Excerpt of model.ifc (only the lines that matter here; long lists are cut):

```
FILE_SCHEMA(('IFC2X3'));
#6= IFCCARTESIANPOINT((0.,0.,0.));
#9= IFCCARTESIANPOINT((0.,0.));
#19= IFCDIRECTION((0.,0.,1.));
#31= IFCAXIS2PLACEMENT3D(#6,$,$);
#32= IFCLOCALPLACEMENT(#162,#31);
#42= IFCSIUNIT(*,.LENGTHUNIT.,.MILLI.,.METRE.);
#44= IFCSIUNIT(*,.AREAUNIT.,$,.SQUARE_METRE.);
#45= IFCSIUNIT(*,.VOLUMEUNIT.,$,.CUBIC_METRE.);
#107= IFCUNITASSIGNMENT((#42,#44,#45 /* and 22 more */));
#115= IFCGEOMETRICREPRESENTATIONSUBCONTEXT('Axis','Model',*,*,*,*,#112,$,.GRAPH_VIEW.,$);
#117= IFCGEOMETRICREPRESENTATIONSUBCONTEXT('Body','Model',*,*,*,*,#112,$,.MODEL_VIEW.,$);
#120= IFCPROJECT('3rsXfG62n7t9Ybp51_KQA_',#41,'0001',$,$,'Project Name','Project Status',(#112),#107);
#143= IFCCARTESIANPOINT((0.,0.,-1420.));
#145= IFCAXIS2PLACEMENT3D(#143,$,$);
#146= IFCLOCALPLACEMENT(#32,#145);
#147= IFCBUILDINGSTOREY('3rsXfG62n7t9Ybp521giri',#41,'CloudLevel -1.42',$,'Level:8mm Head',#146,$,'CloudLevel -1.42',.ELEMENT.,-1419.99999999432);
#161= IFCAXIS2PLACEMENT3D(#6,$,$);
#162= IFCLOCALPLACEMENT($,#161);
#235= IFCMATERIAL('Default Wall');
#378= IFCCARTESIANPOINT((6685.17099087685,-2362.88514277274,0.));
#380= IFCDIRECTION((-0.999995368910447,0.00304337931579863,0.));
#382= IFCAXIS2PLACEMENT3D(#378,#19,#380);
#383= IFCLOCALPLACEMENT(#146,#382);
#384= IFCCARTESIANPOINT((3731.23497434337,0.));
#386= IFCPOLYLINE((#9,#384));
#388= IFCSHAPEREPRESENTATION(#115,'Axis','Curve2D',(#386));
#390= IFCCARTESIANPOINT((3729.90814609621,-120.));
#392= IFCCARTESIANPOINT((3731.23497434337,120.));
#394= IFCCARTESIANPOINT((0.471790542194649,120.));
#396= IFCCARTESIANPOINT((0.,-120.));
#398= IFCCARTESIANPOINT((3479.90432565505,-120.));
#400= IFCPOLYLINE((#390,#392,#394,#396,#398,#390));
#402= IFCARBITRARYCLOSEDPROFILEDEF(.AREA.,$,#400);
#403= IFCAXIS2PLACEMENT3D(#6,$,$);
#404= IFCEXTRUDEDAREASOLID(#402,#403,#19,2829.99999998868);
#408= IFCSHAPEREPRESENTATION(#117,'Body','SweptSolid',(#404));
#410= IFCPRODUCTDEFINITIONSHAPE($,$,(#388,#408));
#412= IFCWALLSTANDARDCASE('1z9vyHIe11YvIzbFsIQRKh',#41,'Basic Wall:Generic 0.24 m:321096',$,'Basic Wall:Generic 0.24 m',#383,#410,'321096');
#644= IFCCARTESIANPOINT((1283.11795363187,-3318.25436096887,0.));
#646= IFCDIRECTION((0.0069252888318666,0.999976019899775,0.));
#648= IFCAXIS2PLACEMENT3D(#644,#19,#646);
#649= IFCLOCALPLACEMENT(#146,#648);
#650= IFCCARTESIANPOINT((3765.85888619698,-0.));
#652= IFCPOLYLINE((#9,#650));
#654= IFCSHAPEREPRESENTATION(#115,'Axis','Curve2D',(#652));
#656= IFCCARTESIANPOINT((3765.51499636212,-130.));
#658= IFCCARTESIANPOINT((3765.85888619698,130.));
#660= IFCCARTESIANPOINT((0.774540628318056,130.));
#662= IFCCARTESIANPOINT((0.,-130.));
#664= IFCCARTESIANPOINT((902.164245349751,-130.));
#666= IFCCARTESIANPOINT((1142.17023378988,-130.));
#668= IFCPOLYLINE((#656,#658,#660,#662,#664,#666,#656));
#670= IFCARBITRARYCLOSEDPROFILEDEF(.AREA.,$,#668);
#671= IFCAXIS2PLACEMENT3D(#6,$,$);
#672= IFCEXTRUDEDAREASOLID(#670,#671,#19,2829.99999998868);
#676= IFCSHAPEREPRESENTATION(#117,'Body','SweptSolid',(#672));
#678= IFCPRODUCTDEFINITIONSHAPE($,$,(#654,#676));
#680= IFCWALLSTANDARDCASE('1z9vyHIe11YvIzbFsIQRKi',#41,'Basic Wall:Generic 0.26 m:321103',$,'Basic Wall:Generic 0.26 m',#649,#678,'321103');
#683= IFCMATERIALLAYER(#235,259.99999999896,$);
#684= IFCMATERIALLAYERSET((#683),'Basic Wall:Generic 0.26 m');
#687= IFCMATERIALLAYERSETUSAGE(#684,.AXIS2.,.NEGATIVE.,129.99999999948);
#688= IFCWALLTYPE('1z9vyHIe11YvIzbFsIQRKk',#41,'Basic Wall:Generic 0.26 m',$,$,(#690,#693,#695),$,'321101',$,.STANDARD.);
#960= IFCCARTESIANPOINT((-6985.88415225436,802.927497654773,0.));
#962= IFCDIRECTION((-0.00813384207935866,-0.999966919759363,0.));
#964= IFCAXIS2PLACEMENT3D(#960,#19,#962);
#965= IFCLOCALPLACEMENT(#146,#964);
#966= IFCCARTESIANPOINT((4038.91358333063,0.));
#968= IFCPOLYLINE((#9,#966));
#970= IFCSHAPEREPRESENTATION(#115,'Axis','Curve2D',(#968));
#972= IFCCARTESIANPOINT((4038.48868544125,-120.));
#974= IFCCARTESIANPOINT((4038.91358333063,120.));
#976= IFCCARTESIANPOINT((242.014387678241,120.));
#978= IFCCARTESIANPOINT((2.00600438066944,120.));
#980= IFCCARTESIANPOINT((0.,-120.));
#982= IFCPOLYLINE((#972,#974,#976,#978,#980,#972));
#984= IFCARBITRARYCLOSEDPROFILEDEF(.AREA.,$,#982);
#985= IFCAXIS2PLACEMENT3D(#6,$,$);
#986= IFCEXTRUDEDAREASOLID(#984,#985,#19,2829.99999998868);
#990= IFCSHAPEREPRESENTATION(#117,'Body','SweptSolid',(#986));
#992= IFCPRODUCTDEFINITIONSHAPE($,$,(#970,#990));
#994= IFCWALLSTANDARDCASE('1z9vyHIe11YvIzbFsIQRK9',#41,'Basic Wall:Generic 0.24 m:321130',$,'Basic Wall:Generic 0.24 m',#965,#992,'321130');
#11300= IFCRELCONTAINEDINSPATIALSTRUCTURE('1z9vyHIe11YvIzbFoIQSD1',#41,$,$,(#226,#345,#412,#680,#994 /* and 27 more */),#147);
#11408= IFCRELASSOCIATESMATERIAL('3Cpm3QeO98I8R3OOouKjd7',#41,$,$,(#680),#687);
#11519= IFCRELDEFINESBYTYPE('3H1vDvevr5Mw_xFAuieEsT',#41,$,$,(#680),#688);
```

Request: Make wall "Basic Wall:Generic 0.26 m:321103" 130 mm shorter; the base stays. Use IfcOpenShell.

```python
import ifcopenshell
import ifcopenshell.geom
import ifcopenshell.util.representation
import ifcopenshell.util.shape
import ifcopenshell.util.unit

model = ifcopenshell.open("model.ifc")
unit_scale = ifcopenshell.util.unit.calculate_unit_scale(model)
settings = ifcopenshell.geom.settings()


def volume(element):
    """Net volume in cubic metres, openings subtracted."""
    shape = ifcopenshell.geom.create_shape(settings, element)
    return ifcopenshell.util.shape.get_volume(shape.geometry)


wall = model.by_guid("1z9vyHIe11YvIzbFsIQRKi")
before = volume(wall)

body = ifcopenshell.util.representation.get_representation(wall, "Model", "Body")
solid = body.Items[0]
old_height = solid.Depth
solid.Depth -= 0.13 / unit_scale
after = volume(wall)

print(f"height {old_height:g} -> {solid.Depth:g}, volume {before:.3f} -> {after:.3f} m3")

model.write("model_edited.ifc")
```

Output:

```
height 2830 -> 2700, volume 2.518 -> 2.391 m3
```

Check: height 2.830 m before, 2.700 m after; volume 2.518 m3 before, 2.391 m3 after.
